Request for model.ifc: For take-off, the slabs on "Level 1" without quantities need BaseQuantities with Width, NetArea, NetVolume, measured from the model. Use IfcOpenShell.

First a look at what the model holds.

```python
import ifcopenshell
import ifcopenshell.util.element
import ifcopenshell.util.unit

model = ifcopenshell.open("model.ifc")
print(model.schema)
for unit_type in ("LENGTHUNIT", "AREAUNIT", "VOLUMEUNIT"):
    print(unit_type, ifcopenshell.util.unit.calculate_unit_scale(model, unit_type))
storey = next(s for s in model.by_type("IfcBuildingStorey") if s.Name == "Level 1")
slabs = [e for e in ifcopenshell.util.element.get_decomposition(storey) if e.is_a("IfcSlab")]
for e in sorted(slabs, key=lambda e: e.id()):
    print(e.id(), e.is_a(), e.Name, list(ifcopenshell.util.element.get_psets(e, qtos_only=True)), sep=" | ")
```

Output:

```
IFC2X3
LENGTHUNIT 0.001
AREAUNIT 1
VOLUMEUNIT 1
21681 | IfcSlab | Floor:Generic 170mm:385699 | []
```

```python
import ifcopenshell
import ifcopenshell.api.pset
import ifcopenshell.geom
import ifcopenshell.util.element
import ifcopenshell.util.shape
import ifcopenshell.util.unit

model = ifcopenshell.open("model.ifc")
unit_scale = ifcopenshell.util.unit.calculate_unit_scale(model)
area_scale = ifcopenshell.util.unit.calculate_unit_scale(model, "AREAUNIT")
volume_scale = ifcopenshell.util.unit.calculate_unit_scale(model, "VOLUMEUNIT")
settings = ifcopenshell.geom.settings()

storey = next(s for s in model.by_type("IfcBuildingStorey") if s.Name == "Level 1")
slabs = [e for e in ifcopenshell.util.element.get_decomposition(storey) if e.is_a("IfcSlab")]

for e in sorted(slabs, key=lambda e: e.id()):
    if ifcopenshell.util.element.get_psets(e, qtos_only=True, should_inherit=False):
        continue
    # Geometry comes back in metres, in the element's own axes.
    shape = ifcopenshell.geom.create_shape(settings, e)
    values = {
        "Width": ifcopenshell.util.shape.get_z(shape.geometry) / unit_scale,
        "NetArea": ifcopenshell.util.shape.get_footprint_area(shape.geometry) / area_scale,
        "NetVolume": ifcopenshell.util.shape.get_volume(shape.geometry) / volume_scale,
    }
    qto = ifcopenshell.api.pset.add_qto(model, product=e, name="BaseQuantities")
    ifcopenshell.api.pset.edit_qto(model, qto=qto, properties=values)
    print(e.id(), {k: round(v, 3) for k, v in values.items()})

model.write("model_edited.ifc")
```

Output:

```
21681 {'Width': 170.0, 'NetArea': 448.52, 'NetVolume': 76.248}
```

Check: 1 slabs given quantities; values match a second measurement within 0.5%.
